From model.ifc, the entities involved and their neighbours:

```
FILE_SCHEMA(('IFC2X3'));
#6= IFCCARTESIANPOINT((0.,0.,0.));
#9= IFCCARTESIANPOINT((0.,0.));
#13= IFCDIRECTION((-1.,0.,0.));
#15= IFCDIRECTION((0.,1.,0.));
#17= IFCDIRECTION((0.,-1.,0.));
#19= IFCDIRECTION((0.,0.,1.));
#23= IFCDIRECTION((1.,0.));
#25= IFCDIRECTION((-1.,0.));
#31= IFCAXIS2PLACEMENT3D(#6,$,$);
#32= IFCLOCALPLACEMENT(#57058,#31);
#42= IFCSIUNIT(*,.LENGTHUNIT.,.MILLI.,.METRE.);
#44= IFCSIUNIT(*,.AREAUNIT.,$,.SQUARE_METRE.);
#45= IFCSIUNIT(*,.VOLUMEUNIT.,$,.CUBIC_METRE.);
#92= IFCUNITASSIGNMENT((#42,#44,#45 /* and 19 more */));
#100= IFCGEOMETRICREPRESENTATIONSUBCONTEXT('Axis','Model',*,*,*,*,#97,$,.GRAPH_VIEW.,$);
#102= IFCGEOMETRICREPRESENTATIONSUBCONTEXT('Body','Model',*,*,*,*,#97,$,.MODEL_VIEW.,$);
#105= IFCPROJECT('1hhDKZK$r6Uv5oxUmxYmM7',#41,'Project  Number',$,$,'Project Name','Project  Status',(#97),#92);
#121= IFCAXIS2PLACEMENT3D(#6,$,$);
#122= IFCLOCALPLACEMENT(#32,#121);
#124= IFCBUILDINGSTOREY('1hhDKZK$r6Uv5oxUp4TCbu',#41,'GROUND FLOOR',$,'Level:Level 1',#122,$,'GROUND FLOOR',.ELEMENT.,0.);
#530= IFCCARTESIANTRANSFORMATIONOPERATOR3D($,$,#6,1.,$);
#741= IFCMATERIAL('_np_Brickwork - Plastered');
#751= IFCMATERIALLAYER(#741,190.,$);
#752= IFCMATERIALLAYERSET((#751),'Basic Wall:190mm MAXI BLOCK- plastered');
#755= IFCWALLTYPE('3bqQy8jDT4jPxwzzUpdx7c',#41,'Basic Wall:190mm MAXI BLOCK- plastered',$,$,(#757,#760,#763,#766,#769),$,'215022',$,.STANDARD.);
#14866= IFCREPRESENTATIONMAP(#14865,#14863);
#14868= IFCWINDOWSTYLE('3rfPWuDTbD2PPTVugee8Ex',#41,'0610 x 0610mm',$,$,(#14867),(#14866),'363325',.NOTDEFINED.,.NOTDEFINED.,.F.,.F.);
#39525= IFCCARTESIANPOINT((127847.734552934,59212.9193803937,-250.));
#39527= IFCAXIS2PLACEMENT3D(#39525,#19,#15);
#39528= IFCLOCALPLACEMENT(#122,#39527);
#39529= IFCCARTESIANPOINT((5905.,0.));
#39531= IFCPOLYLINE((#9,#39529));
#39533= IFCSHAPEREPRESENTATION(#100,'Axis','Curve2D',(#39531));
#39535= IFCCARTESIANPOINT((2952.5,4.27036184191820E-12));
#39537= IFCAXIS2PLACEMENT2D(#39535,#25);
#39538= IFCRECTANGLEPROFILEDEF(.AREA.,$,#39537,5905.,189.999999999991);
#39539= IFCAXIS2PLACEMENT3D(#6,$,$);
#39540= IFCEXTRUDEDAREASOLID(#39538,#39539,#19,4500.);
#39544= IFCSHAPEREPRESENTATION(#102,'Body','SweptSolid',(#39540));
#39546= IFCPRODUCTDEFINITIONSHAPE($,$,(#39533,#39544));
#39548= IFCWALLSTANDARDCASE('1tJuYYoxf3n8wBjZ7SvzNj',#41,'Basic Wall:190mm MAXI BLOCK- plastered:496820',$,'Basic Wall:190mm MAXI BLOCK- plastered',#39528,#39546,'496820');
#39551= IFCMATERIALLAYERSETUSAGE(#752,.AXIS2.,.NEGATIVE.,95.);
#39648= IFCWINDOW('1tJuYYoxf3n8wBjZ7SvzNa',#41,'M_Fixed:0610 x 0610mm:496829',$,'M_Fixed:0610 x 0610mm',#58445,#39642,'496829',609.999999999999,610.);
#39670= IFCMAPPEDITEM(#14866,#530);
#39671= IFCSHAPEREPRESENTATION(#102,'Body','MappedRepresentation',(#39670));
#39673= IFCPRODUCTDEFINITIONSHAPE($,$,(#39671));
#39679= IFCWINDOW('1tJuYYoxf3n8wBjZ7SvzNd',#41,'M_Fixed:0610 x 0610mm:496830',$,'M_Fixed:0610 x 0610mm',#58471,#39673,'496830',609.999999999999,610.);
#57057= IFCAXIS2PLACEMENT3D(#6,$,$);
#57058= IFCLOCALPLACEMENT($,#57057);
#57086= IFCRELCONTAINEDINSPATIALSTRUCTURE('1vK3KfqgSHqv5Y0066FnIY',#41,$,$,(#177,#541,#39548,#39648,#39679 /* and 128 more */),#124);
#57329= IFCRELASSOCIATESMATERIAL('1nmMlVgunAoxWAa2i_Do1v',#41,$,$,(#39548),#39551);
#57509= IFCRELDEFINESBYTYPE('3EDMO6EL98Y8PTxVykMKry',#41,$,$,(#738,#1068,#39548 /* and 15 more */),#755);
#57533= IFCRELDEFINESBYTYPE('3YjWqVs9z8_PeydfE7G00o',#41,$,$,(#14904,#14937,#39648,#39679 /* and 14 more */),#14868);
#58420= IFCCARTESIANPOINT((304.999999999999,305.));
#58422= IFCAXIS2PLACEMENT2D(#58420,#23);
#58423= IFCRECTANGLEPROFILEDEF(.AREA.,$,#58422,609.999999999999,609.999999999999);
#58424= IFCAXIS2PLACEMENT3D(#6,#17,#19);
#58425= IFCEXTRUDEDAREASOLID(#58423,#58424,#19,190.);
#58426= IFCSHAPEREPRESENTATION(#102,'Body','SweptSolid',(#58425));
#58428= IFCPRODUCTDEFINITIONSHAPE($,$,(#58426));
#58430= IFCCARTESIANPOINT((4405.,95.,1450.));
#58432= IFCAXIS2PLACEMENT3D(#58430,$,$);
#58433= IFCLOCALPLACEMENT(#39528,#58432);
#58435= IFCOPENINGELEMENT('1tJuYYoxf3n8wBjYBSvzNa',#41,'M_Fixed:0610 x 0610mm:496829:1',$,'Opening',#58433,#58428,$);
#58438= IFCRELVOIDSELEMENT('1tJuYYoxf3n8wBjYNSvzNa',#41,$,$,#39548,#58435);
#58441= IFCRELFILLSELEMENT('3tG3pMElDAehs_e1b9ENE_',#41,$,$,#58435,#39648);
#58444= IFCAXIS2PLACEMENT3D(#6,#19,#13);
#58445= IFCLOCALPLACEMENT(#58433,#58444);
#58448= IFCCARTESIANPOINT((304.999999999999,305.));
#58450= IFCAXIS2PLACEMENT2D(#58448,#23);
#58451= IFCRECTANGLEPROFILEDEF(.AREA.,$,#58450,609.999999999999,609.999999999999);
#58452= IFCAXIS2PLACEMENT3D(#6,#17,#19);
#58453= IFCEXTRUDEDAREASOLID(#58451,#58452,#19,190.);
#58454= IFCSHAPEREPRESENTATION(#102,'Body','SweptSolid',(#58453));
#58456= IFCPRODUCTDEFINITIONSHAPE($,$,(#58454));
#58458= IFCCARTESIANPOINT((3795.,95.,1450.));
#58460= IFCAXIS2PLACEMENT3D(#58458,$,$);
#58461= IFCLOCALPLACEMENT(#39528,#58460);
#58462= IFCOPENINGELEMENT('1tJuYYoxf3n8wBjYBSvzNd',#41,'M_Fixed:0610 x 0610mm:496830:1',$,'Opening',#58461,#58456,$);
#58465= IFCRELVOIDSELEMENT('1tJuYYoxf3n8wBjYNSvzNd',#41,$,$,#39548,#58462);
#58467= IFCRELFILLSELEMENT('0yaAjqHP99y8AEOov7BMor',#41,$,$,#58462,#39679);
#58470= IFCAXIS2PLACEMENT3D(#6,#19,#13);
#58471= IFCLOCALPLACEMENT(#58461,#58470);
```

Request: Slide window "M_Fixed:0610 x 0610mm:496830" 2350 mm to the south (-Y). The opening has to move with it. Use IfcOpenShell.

```python
import ifcopenshell
import ifcopenshell.api.geometry
import ifcopenshell.util.placement
import ifcopenshell.util.unit

model = ifcopenshell.open("model.ifc")
unit_scale = ifcopenshell.util.unit.calculate_unit_scale(model)

window = model.by_id(39679)
opening = window.FillsVoids[0].RelatingOpeningElement
wall = opening.VoidsElements[0].RelatingBuildingElement

wall_matrix = ifcopenshell.util.placement.get_local_placement(wall.ObjectPlacement)
shift = wall_matrix[:3, 0] * -2.35 / unit_scale
before = ifcopenshell.util.placement.get_local_placement(window.ObjectPlacement)[:3, 3].copy()

# The window is placed relative to its opening, so it follows when the opening moves.
matrix = ifcopenshell.util.placement.get_local_placement(opening.ObjectPlacement)
matrix[:3, 3] += shift
ifcopenshell.api.geometry.edit_object_placement(
    model, product=opening, matrix=matrix, is_si=False, should_transform_children=True
)

after = ifcopenshell.util.placement.get_local_placement(window.ObjectPlacement)[:3, 3]
print("window moved by", (after - before).round(3) + 0.0)

model.write("model_rev.ifc")
```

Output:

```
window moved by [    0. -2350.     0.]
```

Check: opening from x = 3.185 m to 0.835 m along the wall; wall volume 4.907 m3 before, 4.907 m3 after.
